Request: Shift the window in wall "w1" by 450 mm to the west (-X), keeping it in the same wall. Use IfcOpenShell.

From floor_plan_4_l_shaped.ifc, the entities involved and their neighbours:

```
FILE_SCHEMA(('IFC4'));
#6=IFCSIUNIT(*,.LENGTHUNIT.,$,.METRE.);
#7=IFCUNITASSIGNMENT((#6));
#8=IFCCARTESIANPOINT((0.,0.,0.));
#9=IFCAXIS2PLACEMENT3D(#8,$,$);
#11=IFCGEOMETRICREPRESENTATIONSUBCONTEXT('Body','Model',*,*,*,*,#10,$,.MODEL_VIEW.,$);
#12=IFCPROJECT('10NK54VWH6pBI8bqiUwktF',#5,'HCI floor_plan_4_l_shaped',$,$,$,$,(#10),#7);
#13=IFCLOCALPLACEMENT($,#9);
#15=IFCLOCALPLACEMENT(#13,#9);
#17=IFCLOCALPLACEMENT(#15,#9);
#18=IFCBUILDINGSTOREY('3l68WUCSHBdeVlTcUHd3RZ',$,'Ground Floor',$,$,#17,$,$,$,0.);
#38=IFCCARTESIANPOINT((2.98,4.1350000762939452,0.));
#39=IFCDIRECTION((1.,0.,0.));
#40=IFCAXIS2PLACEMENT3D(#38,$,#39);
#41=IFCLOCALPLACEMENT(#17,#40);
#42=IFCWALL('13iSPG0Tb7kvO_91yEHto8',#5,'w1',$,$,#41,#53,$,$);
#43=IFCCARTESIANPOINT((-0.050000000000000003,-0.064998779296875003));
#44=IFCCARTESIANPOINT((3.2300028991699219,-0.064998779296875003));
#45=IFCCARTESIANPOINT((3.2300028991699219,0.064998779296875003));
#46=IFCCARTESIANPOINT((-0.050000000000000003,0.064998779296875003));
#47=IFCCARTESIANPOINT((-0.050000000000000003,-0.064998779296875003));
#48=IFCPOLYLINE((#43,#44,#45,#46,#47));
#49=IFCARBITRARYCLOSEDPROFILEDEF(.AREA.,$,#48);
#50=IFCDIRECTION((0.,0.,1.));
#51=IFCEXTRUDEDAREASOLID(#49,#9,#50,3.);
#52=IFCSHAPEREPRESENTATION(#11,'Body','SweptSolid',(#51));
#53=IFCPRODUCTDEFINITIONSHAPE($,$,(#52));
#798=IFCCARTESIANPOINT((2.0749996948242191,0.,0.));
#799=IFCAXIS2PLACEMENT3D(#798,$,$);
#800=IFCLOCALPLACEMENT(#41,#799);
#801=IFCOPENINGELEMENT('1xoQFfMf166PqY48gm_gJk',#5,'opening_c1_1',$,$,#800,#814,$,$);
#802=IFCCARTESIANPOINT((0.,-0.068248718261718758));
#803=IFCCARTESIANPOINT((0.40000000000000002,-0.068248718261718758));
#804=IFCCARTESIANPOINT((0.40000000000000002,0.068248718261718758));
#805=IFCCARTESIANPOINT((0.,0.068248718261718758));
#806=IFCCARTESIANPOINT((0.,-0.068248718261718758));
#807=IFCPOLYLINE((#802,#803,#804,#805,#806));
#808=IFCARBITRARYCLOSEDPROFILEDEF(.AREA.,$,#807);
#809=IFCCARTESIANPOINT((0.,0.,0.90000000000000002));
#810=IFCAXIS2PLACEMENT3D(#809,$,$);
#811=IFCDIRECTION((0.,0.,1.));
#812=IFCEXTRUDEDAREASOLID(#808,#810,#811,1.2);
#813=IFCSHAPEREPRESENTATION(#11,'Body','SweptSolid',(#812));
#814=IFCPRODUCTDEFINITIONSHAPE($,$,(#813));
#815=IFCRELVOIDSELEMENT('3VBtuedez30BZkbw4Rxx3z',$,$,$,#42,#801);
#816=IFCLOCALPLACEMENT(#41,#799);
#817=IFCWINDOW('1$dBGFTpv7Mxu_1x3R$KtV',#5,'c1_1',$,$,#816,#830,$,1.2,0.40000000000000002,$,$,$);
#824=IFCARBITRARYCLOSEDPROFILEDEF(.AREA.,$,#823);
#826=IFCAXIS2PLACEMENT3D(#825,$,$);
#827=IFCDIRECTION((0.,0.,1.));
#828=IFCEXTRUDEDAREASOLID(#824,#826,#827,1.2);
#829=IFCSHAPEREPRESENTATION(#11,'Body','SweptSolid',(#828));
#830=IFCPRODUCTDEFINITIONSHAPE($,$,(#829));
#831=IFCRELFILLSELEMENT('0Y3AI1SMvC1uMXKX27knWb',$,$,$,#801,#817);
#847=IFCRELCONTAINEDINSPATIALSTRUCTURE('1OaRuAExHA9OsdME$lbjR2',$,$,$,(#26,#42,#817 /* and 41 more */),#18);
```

```python
import ifcopenshell
import ifcopenshell.api.geometry
import ifcopenshell.util.placement
import ifcopenshell.util.unit

model = ifcopenshell.open("floor_plan_4_l_shaped.ifc")
unit_scale = ifcopenshell.util.unit.calculate_unit_scale(model)

window = model.by_id(817)
opening = window.FillsVoids[0].RelatingOpeningElement
wall = opening.VoidsElements[0].RelatingBuildingElement

wall_matrix = ifcopenshell.util.placement.get_local_placement(wall.ObjectPlacement)
shift = wall_matrix[:3, 0] * -0.45 / unit_scale
before = ifcopenshell.util.placement.get_local_placement(window.ObjectPlacement)[:3, 3].copy()

# The window is not placed relative to its opening, so move both.
for product in (opening, window):
    matrix = ifcopenshell.util.placement.get_local_placement(product.ObjectPlacement)
    matrix[:3, 3] += shift
    ifcopenshell.api.geometry.edit_object_placement(model, product=product, matrix=matrix, is_si=False)

after = ifcopenshell.util.placement.get_local_placement(window.ObjectPlacement)[:3, 3]
print("window moved by", (after - before).round(3) + 0.0)

model.write("floor_plan_4_l_shaped_rev.ifc")
```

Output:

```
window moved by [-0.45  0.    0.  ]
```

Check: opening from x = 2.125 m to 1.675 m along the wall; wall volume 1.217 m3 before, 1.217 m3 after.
